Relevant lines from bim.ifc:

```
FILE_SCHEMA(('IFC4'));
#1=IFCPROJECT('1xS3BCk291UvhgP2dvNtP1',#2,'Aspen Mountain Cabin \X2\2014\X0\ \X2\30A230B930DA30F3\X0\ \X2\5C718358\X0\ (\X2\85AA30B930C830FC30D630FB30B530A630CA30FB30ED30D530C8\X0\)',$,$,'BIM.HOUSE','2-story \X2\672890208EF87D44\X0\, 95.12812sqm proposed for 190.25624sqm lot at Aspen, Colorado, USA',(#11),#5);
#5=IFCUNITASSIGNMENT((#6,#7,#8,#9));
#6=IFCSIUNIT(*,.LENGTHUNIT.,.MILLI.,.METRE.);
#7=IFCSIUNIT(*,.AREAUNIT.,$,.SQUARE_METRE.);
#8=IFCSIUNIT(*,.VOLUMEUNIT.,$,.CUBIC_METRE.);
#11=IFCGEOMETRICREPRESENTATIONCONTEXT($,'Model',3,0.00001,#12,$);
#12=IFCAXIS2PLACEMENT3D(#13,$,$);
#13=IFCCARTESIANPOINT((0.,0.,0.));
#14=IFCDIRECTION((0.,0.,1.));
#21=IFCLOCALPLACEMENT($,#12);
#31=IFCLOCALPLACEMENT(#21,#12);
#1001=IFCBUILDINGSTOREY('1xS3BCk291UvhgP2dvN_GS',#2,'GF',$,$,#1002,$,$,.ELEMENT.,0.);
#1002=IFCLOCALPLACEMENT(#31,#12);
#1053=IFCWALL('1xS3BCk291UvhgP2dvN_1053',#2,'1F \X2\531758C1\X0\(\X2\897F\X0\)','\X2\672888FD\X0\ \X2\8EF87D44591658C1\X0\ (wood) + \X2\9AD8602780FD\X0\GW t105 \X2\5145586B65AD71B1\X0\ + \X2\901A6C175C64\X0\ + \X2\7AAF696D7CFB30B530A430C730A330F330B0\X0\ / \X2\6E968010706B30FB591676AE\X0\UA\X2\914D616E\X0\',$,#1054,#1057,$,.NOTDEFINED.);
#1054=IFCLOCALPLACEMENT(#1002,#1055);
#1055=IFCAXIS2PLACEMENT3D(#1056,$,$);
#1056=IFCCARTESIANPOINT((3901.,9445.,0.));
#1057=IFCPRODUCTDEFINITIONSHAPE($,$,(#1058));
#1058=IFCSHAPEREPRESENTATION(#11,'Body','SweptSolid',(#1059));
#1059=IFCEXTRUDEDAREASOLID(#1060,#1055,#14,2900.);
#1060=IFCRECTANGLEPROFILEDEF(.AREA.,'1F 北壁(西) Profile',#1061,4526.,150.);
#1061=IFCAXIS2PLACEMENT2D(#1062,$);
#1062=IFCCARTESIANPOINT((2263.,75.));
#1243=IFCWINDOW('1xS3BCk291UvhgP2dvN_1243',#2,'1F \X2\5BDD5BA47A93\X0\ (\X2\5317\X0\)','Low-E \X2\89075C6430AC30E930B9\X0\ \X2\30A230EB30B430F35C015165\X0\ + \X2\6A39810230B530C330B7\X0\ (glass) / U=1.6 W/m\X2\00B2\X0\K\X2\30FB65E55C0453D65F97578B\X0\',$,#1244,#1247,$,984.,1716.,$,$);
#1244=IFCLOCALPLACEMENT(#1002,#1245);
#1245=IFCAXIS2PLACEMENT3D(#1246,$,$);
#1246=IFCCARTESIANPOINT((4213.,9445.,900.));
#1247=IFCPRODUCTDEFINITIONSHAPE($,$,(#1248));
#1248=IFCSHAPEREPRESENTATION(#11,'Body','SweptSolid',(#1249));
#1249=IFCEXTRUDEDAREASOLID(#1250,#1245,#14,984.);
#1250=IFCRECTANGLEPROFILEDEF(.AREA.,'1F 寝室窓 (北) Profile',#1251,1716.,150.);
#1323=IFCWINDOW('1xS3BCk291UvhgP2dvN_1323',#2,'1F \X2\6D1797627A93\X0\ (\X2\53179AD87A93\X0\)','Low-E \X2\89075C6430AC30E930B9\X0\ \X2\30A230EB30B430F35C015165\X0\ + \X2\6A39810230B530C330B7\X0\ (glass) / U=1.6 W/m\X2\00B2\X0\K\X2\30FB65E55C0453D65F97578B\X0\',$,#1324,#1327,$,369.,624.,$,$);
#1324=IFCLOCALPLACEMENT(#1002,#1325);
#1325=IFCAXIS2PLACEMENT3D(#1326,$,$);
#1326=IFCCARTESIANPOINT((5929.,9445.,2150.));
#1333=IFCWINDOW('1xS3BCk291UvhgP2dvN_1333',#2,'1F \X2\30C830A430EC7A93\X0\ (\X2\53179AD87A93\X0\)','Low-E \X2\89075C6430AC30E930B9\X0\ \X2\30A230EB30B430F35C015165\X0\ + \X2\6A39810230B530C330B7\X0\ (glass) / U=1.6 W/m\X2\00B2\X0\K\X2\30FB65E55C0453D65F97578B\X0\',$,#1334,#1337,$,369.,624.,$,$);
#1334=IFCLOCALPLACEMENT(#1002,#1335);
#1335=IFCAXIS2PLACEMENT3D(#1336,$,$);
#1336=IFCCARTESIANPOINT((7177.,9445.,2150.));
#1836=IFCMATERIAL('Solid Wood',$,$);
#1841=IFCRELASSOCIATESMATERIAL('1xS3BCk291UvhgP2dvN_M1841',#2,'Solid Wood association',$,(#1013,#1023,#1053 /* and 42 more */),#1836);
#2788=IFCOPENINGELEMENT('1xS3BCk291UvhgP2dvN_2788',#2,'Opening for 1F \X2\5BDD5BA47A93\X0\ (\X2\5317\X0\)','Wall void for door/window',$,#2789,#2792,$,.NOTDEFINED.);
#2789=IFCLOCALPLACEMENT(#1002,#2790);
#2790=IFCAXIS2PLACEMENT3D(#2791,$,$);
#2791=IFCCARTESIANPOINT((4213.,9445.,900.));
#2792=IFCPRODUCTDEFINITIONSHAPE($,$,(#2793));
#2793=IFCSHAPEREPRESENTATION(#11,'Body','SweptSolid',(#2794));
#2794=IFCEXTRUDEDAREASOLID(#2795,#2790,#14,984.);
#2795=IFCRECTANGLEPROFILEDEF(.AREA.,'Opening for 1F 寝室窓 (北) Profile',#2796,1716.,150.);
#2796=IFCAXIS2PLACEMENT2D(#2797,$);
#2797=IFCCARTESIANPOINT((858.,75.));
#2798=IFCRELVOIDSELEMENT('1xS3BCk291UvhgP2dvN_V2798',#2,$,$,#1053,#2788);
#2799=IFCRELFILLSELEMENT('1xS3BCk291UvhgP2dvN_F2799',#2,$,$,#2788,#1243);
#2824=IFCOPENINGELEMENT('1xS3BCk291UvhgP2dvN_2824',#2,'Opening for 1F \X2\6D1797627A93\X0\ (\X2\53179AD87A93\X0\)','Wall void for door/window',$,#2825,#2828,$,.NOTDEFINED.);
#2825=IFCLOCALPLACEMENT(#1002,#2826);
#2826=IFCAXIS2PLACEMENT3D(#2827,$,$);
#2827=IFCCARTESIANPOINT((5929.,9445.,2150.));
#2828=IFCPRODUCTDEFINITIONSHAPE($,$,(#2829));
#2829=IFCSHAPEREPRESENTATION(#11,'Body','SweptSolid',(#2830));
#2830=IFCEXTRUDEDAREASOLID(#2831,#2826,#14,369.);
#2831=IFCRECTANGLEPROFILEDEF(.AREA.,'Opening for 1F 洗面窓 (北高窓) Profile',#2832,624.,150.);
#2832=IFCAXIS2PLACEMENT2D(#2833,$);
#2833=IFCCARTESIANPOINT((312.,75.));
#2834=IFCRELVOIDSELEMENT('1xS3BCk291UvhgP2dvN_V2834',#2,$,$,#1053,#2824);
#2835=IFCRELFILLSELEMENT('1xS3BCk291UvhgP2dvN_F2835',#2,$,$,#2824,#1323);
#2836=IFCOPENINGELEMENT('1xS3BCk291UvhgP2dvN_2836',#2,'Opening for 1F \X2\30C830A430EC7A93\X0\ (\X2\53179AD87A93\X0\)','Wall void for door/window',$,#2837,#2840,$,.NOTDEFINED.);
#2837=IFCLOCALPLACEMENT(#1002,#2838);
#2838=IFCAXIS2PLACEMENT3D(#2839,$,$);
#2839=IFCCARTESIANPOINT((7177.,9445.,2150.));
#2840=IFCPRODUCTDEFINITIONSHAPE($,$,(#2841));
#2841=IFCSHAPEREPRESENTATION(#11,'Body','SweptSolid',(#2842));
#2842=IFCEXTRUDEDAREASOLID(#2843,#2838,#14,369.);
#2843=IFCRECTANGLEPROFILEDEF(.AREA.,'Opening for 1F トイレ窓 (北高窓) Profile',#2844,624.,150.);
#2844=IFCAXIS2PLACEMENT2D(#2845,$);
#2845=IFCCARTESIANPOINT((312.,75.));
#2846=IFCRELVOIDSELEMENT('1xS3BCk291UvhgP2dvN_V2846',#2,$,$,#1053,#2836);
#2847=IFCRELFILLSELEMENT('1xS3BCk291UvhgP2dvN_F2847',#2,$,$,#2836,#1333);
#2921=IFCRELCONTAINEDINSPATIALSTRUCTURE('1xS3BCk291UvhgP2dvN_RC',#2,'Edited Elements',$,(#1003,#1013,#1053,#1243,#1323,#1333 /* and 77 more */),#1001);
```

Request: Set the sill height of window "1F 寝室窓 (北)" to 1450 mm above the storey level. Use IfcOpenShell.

```python
import numpy as np
import ifcopenshell
import ifcopenshell.api.geometry
import ifcopenshell.geom
import ifcopenshell.util.element
import ifcopenshell.util.placement
import ifcopenshell.util.shape
import ifcopenshell.util.unit

model = ifcopenshell.open("bim.ifc")
unit_scale = ifcopenshell.util.unit.calculate_unit_scale(model)

window = model.by_guid("1xS3BCk291UvhgP2dvN_1243")
opening = window.FillsVoids[0].RelatingOpeningElement
storey = ifcopenshell.util.element.get_container(window, ifc_class="IfcBuildingStorey")
level = ifcopenshell.util.placement.get_local_placement(storey.ObjectPlacement)[2, 3]

# The opening's origin need not be at the sill, so measure its lowest point.
shape = ifcopenshell.geom.create_shape(ifcopenshell.geom.settings(), opening)
bottom = ifcopenshell.util.shape.get_shape_bottom_elevation(shape, shape.geometry) / unit_scale
dz = level + 1.45 / unit_scale - bottom

shift = np.array([0.0, 0.0, dz])
# The window is not placed relative to its opening, so move both.
for product in (opening, window):
    matrix = ifcopenshell.util.placement.get_local_placement(product.ObjectPlacement)
    matrix[:3, 3] += shift
    ifcopenshell.api.geometry.edit_object_placement(model, product=product, matrix=matrix, is_si=False)

print(f"moved by {dz * unit_scale:+.3f} m")

model.write("bim_rev.ifc")
```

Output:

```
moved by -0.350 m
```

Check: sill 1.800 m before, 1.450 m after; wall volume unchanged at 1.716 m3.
